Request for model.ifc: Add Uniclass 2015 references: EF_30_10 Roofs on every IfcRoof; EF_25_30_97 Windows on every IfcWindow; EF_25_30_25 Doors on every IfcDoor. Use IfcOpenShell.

First a look at what the model holds.

```python
import ifcopenshell

model = ifcopenshell.open("model.ifc")
print(model.schema)
print("classifications:", [c.Name for c in model.by_type("IfcClassification")])
for ifc_class in ("IfcDoor", "IfcRoof", "IfcStair", "IfcWall", "IfcWindow"):
    print(ifc_class, len(model.by_type(ifc_class)))
```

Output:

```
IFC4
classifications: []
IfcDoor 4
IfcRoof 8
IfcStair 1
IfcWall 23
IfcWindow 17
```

```python
import ifcopenshell
import ifcopenshell.api.classification

model = ifcopenshell.open("model.ifc")

system = ifcopenshell.api.classification.add_classification(model, classification="Uniclass 2015")

codes = {
    "IfcRoof": ("EF_30_10", "Roofs"),
    "IfcWindow": ("EF_25_30_97", "Windows"),
    "IfcDoor": ("EF_25_30_25", "Doors"),
}
for ifc_class, (code, name) in codes.items():
    products = model.by_type(ifc_class)
    ifcopenshell.api.classification.add_reference(
        model, products=products, classification=system, identification=code, name=name
    )
    print(code, len(products))

model.write("model_updated.ifc")
```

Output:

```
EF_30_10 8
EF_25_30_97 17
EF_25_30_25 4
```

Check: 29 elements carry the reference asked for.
